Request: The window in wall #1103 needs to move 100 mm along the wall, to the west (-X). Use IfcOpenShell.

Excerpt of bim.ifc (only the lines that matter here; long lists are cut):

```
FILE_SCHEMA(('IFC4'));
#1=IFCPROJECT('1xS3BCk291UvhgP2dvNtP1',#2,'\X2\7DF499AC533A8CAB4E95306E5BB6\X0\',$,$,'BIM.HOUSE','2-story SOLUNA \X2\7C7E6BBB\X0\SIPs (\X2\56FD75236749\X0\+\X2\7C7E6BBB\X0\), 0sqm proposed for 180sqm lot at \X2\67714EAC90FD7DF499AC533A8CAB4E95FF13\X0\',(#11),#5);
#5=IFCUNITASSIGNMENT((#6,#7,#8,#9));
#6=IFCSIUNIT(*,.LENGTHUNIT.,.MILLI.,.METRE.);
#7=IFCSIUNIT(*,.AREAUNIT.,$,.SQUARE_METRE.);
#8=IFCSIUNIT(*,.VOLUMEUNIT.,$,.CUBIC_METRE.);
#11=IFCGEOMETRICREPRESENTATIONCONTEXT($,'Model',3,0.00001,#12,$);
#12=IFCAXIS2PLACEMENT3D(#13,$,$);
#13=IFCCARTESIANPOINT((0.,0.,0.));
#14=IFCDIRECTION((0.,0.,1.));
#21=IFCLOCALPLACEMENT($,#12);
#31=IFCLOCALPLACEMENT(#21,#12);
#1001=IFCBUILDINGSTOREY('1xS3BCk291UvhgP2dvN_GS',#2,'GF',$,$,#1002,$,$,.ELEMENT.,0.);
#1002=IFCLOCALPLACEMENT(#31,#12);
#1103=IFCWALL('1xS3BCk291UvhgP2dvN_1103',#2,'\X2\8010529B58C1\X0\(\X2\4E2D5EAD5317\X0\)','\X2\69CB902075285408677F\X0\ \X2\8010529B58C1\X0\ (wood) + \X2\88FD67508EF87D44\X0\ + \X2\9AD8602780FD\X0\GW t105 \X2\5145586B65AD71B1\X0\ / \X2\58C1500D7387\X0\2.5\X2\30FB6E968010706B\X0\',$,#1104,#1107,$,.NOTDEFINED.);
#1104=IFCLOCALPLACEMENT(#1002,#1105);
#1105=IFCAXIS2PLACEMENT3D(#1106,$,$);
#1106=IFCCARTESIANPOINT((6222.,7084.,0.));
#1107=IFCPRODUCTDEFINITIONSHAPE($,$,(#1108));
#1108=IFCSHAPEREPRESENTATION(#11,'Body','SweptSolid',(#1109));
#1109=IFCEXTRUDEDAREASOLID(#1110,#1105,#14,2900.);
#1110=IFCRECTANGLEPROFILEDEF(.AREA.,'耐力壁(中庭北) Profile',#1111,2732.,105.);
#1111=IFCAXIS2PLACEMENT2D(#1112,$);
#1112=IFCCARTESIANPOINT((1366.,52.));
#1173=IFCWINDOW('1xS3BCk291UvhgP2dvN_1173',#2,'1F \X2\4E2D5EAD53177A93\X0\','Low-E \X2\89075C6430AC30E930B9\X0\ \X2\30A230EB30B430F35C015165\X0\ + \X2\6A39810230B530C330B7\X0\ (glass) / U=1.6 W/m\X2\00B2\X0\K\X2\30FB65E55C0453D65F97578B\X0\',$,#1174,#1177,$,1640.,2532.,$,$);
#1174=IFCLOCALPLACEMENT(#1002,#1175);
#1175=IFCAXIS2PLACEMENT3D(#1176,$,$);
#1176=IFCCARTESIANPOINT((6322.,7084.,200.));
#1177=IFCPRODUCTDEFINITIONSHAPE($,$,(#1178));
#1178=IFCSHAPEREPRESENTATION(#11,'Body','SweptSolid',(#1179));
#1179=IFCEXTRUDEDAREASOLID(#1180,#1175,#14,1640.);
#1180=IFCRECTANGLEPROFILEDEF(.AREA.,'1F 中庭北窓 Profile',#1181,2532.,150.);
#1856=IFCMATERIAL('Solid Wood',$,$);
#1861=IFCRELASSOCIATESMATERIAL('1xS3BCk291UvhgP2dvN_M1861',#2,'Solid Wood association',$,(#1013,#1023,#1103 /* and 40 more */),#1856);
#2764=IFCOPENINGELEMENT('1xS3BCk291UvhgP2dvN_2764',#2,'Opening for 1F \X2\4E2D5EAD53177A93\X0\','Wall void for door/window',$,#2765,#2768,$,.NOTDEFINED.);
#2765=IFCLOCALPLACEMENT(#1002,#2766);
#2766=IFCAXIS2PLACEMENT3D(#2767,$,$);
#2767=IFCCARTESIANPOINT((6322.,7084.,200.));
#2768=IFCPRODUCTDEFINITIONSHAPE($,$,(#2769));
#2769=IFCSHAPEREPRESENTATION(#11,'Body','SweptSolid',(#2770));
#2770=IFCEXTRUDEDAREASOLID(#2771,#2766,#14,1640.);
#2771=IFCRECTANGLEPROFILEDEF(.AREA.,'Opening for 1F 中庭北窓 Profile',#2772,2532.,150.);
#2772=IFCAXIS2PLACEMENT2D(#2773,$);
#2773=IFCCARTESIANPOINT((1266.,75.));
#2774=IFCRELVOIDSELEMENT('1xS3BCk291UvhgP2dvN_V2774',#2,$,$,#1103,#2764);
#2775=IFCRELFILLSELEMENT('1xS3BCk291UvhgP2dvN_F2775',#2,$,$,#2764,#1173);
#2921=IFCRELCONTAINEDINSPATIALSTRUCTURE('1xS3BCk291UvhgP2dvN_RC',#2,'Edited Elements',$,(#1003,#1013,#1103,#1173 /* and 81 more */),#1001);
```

```python
import ifcopenshell
import ifcopenshell.api.geometry
import ifcopenshell.util.placement
import ifcopenshell.util.unit

model = ifcopenshell.open("bim.ifc")
unit_scale = ifcopenshell.util.unit.calculate_unit_scale(model)

window = model.by_id(1173)
opening = window.FillsVoids[0].RelatingOpeningElement
wall = opening.VoidsElements[0].RelatingBuildingElement

wall_matrix = ifcopenshell.util.placement.get_local_placement(wall.ObjectPlacement)
shift = wall_matrix[:3, 0] * -0.1 / unit_scale
before = ifcopenshell.util.placement.get_local_placement(window.ObjectPlacement)[:3, 3].copy()

# The window is not placed relative to its opening, so move both.
for product in (opening, window):
    matrix = ifcopenshell.util.placement.get_local_placement(product.ObjectPlacement)
    matrix[:3, 3] += shift
    ifcopenshell.api.geometry.edit_object_placement(model, product=product, matrix=matrix, is_si=False)

after = ifcopenshell.util.placement.get_local_placement(window.ObjectPlacement)[:3, 3]
print("window moved by", (after - before).round(3) + 0.0)

model.write("bim_rev.ifc")
```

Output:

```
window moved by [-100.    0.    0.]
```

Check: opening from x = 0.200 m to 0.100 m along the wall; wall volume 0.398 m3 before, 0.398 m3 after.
